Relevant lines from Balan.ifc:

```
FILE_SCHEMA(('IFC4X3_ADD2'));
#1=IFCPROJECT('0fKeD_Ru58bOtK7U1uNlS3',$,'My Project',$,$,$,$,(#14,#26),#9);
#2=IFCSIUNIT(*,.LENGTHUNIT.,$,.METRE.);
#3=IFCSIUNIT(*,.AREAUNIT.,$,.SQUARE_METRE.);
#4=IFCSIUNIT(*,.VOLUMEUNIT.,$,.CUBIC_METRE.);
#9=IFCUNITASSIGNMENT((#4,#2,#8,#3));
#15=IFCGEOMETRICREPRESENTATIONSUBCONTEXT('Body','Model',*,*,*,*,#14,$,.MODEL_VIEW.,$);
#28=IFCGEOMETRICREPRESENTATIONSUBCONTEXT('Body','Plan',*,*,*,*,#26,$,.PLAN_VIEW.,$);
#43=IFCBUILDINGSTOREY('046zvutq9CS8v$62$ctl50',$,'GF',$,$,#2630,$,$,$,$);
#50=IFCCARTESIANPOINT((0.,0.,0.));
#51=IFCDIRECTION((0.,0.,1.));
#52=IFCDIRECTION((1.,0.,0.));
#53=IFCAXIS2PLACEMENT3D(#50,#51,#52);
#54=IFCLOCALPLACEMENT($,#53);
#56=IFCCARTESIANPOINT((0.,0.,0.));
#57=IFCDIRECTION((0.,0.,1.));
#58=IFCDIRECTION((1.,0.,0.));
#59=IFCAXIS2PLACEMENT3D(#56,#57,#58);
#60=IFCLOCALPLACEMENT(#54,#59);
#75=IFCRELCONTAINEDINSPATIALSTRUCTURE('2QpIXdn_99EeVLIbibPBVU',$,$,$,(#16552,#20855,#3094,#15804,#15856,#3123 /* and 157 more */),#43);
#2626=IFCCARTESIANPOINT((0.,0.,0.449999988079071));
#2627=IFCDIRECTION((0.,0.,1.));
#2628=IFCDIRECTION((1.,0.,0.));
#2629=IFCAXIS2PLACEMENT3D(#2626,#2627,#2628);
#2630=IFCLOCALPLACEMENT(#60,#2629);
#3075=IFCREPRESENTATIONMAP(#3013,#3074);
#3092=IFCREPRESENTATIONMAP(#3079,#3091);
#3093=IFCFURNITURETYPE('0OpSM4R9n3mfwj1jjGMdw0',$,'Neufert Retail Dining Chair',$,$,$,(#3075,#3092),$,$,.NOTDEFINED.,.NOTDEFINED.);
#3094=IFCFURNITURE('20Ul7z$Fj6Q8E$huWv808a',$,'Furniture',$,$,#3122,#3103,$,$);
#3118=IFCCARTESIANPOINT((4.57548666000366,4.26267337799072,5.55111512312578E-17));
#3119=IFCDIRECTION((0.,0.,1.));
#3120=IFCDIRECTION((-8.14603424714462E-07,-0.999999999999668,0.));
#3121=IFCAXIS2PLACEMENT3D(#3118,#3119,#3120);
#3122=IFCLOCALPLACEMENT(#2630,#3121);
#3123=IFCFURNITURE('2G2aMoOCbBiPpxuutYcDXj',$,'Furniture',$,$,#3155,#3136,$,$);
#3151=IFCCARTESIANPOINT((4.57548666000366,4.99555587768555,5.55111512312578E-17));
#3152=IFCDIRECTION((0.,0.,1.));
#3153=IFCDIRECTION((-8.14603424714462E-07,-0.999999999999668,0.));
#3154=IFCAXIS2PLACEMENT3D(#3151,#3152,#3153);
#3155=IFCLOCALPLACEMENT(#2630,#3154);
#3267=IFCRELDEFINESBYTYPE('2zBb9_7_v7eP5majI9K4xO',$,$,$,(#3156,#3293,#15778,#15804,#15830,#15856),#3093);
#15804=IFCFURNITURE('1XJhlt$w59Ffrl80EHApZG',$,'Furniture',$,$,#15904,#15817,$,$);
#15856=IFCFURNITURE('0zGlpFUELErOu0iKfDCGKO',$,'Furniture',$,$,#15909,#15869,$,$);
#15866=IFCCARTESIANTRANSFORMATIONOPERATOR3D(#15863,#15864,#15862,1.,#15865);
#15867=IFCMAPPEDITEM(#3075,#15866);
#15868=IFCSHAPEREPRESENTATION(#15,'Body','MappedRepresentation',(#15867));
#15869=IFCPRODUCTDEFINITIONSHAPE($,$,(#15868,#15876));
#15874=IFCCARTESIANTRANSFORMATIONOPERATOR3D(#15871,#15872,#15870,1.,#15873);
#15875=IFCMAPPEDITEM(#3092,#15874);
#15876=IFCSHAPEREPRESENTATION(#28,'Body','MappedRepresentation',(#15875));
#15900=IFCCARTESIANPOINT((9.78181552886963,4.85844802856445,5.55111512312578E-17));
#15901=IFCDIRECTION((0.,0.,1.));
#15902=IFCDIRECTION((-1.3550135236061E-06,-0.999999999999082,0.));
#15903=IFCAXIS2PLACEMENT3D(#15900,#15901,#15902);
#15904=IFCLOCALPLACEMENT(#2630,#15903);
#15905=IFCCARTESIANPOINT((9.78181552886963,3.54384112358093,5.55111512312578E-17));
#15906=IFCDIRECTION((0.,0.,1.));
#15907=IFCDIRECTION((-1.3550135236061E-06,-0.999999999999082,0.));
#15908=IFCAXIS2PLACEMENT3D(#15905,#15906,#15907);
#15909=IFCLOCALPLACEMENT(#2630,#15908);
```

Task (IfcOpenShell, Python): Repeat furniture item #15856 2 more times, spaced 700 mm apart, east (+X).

```python
import numpy as np
import ifcopenshell
import ifcopenshell.api.geometry
import ifcopenshell.api.root
import ifcopenshell.util.element
import ifcopenshell.util.placement
import ifcopenshell.util.unit

model = ifcopenshell.open("Balan.ifc")
unit_scale = ifcopenshell.util.unit.calculate_unit_scale(model)

source = model.by_id(15856)
base = ifcopenshell.util.placement.get_local_placement(source.ObjectPlacement)
step = np.array([1.0, 0.0, 0.0]) * 0.7 / unit_scale

for i in range(1, 3):
    copy = ifcopenshell.api.root.copy_class(model, product=source)
    copy.Representation = ifcopenshell.util.element.copy_deep(
        model, source.Representation, exclude=["IfcGeometricRepresentationContext", "IfcRepresentationMap"]
    )
    matrix = base.copy()
    matrix[:3, 3] += i * step
    print("added at", matrix[:3, 3].round(3) + 0.0)
    ifcopenshell.api.geometry.edit_object_placement(model, product=copy, matrix=matrix, is_si=False)

model.write("Balan_updated.ifc")
```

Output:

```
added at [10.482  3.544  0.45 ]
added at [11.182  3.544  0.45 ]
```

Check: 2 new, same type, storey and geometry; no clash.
